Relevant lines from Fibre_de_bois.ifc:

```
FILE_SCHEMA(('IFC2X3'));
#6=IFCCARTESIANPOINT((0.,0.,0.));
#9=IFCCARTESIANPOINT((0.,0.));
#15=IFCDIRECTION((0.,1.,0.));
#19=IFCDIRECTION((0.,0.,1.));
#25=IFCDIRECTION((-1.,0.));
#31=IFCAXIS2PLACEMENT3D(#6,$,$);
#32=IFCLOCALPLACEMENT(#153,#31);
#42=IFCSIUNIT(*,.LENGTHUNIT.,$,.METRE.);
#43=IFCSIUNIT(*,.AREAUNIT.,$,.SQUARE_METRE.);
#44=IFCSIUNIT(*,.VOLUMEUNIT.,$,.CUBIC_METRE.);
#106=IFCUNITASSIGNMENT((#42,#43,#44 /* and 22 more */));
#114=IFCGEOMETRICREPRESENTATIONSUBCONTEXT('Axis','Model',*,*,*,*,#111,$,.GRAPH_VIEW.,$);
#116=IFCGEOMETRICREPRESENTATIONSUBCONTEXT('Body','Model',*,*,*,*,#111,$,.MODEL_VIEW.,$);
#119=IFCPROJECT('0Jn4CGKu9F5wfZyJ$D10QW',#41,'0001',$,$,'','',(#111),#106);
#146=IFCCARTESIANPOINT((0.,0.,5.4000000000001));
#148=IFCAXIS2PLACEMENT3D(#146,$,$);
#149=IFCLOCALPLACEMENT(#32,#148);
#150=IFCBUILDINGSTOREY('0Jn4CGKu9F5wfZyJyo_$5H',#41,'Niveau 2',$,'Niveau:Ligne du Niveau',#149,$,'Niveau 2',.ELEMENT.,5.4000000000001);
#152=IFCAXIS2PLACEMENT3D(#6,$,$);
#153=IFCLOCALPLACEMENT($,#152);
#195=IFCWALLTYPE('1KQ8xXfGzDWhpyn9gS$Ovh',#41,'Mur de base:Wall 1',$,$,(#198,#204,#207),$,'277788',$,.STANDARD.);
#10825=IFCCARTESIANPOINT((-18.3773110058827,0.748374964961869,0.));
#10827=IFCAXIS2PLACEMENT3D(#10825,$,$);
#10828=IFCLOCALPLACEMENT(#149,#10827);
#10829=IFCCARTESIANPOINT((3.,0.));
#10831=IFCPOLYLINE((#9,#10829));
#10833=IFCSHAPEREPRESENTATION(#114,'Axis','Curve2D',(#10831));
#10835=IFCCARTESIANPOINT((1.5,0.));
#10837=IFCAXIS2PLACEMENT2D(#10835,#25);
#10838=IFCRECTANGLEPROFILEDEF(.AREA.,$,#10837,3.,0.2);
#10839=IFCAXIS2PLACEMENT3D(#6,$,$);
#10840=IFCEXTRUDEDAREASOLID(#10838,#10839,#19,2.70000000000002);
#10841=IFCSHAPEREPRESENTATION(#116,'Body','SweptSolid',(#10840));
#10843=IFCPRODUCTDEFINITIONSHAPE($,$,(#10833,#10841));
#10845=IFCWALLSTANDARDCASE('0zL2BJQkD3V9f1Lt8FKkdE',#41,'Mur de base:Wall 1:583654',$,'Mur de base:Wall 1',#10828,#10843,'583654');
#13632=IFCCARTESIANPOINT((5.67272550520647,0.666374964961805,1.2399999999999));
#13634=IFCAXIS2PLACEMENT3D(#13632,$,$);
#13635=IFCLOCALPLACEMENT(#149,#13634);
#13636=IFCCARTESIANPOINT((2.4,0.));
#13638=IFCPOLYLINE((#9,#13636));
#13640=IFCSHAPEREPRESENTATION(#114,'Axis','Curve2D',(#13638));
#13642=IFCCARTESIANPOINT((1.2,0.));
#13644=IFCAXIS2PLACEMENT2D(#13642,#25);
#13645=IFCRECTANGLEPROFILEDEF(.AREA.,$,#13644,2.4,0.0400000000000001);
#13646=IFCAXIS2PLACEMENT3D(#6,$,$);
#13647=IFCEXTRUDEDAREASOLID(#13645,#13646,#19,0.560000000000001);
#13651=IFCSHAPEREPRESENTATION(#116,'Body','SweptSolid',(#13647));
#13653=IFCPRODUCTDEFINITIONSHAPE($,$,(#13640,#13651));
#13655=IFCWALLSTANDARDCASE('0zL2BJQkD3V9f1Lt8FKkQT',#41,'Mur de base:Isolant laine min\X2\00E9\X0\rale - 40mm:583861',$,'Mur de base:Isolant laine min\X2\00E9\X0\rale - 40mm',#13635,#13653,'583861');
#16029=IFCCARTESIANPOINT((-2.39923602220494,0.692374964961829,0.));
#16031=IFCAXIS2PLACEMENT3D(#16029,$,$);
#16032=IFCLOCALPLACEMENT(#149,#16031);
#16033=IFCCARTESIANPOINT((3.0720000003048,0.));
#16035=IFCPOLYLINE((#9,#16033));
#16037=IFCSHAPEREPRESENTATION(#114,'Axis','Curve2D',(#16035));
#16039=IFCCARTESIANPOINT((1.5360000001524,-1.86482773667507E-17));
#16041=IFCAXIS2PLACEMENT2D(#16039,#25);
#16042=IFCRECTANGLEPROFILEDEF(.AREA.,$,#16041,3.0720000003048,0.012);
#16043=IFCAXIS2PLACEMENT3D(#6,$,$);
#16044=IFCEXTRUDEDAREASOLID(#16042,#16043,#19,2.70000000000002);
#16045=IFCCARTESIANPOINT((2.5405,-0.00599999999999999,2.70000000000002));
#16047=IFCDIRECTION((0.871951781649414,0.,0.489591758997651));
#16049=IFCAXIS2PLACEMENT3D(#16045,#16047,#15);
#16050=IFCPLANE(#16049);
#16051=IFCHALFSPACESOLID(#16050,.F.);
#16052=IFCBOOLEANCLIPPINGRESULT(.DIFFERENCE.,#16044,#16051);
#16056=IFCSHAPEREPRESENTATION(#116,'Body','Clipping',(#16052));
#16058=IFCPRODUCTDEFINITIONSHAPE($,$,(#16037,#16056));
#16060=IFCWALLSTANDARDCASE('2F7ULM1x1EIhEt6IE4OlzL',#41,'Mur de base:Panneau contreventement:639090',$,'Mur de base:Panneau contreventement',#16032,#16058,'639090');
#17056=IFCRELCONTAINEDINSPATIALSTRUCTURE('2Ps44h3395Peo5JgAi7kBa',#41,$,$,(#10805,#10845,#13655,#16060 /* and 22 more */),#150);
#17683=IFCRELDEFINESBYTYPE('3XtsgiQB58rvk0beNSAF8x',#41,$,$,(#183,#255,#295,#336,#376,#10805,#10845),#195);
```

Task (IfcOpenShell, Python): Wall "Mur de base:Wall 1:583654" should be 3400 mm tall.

```python
import ifcopenshell
import ifcopenshell.geom
import ifcopenshell.util.representation
import ifcopenshell.util.shape

model = ifcopenshell.open("Fibre_de_bois.ifc")
settings = ifcopenshell.geom.settings()


def volume(element):
    """Net volume in cubic metres, openings subtracted."""
    shape = ifcopenshell.geom.create_shape(settings, element)
    return ifcopenshell.util.shape.get_volume(shape.geometry)


wall = model.by_guid("0zL2BJQkD3V9f1Lt8FKkdE")
before = volume(wall)

body = ifcopenshell.util.representation.get_representation(wall, "Model", "Body")
solid = body.Items[0]
old_height = solid.Depth
solid.Depth = 3.4
after = volume(wall)

print(f"height {old_height:g} -> {solid.Depth:g}, volume {before:.3f} -> {after:.3f} m3")

model.write("Fibre_de_bois_updated.ifc")
```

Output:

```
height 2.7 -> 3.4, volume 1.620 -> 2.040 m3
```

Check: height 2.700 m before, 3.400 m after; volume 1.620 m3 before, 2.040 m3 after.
